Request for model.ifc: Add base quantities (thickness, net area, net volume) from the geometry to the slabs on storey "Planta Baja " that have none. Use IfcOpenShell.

First a look at what the model holds.

```python
import ifcopenshell
import ifcopenshell.util.element
import ifcopenshell.util.unit

model = ifcopenshell.open("model.ifc")
print(model.schema)
for unit_type in ("LENGTHUNIT", "AREAUNIT", "VOLUMEUNIT"):
    print(unit_type, ifcopenshell.util.unit.calculate_unit_scale(model, unit_type))
storey = next(s for s in model.by_type("IfcBuildingStorey") if s.Name == "Planta Baja ")
slabs = [e for e in ifcopenshell.util.element.get_decomposition(storey) if e.is_a("IfcSlab")]
for e in sorted(slabs, key=lambda e: e.id()):
    print(e.id(), e.is_a(), e.Name, list(ifcopenshell.util.element.get_psets(e, qtos_only=True)), sep=" | ")
```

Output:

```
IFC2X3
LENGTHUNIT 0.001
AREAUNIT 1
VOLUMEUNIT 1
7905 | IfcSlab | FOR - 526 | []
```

```python
import ifcopenshell
import ifcopenshell.api.pset
import ifcopenshell.geom
import ifcopenshell.util.element
import ifcopenshell.util.shape
import ifcopenshell.util.unit

model = ifcopenshell.open("model.ifc")
unit_scale = ifcopenshell.util.unit.calculate_unit_scale(model)
area_scale = ifcopenshell.util.unit.calculate_unit_scale(model, "AREAUNIT")
volume_scale = ifcopenshell.util.unit.calculate_unit_scale(model, "VOLUMEUNIT")
settings = ifcopenshell.geom.settings()

storey = next(s for s in model.by_type("IfcBuildingStorey") if s.Name == "Planta Baja ")
slabs = [e for e in ifcopenshell.util.element.get_decomposition(storey) if e.is_a("IfcSlab")]

for e in sorted(slabs, key=lambda e: e.id()):
    if ifcopenshell.util.element.get_psets(e, qtos_only=True, should_inherit=False):
        continue
    # Geometry comes back in metres, in the element's own axes.
    shape = ifcopenshell.geom.create_shape(settings, e)
    values = {
        "Width": ifcopenshell.util.shape.get_z(shape.geometry) / unit_scale,
        "NetArea": ifcopenshell.util.shape.get_footprint_area(shape.geometry) / area_scale,
        "NetVolume": ifcopenshell.util.shape.get_volume(shape.geometry) / volume_scale,
    }
    qto = ifcopenshell.api.pset.add_qto(model, product=e, name="BaseQuantities")
    ifcopenshell.api.pset.edit_qto(model, qto=qto, properties=values)
    print(e.id(), {k: round(v, 3) for k, v in values.items()})

model.write("model_v2.ifc")
```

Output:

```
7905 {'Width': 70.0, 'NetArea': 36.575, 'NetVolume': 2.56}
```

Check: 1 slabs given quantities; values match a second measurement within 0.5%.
